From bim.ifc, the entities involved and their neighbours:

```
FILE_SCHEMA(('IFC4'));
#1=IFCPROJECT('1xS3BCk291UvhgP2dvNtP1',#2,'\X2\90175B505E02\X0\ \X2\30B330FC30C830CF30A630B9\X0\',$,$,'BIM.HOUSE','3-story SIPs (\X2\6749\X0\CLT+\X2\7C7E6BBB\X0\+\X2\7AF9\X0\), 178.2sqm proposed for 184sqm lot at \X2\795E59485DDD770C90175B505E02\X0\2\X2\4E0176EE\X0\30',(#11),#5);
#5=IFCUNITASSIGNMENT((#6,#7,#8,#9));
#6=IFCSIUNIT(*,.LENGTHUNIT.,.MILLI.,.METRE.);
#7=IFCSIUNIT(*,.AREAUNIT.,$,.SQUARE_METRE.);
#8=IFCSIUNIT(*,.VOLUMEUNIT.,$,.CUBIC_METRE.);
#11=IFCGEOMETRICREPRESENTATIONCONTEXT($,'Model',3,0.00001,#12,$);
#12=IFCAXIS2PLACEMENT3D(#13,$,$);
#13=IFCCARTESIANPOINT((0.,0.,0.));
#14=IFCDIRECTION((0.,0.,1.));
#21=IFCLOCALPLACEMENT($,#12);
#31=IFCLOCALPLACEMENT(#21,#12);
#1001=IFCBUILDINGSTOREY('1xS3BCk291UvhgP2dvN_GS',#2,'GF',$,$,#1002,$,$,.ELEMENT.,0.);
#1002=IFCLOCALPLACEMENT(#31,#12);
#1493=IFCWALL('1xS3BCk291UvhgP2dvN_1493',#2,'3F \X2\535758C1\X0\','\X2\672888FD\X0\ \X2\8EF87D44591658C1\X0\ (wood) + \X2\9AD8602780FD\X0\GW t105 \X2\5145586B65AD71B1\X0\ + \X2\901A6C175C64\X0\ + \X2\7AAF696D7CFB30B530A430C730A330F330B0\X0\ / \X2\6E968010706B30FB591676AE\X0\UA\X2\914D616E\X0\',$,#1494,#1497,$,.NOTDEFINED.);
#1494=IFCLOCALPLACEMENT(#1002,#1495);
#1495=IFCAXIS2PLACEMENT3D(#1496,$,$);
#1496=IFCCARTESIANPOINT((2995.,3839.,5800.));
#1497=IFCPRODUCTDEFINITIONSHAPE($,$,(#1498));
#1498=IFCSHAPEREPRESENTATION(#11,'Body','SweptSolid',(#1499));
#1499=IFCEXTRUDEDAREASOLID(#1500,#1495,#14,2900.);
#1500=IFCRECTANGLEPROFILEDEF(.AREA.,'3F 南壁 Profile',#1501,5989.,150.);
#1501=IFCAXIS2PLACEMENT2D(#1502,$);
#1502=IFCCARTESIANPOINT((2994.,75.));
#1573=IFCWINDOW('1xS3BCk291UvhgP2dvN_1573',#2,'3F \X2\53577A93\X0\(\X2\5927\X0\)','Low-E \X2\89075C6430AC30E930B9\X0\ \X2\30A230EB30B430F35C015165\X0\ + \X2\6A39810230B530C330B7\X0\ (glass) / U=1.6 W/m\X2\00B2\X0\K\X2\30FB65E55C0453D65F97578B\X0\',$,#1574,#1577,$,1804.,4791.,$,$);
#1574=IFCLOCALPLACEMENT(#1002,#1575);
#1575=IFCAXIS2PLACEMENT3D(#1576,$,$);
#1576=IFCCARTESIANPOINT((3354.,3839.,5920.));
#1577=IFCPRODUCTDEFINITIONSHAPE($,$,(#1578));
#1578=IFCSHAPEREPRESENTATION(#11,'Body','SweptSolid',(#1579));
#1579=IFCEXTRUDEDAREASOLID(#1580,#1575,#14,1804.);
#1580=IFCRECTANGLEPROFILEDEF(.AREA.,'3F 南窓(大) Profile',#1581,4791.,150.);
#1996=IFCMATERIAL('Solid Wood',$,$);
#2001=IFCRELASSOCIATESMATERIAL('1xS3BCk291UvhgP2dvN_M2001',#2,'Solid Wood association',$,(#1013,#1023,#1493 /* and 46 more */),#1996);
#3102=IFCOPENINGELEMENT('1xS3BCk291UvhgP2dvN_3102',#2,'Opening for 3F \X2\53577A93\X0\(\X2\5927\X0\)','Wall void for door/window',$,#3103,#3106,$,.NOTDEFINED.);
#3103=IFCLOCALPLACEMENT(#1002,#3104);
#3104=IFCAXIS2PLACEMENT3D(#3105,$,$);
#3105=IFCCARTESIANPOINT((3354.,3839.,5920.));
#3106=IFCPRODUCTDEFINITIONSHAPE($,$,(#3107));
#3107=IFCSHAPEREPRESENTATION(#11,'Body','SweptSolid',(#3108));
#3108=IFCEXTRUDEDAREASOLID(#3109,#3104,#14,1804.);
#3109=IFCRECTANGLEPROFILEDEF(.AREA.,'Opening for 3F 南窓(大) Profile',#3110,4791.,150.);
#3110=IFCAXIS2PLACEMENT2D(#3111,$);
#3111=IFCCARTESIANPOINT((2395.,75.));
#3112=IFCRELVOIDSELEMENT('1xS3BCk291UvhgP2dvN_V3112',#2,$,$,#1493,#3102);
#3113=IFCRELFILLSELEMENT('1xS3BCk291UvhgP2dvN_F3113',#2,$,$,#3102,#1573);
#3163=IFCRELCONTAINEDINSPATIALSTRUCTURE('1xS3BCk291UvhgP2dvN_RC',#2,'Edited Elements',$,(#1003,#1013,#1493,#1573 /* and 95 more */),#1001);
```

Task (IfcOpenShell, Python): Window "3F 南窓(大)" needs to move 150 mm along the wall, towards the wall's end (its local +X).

```python
import ifcopenshell
import ifcopenshell.api.geometry
import ifcopenshell.util.placement
import ifcopenshell.util.unit

model = ifcopenshell.open("bim.ifc")
unit_scale = ifcopenshell.util.unit.calculate_unit_scale(model)

window = model.by_guid("1xS3BCk291UvhgP2dvN_1573")
opening = window.FillsVoids[0].RelatingOpeningElement
wall = opening.VoidsElements[0].RelatingBuildingElement

wall_matrix = ifcopenshell.util.placement.get_local_placement(wall.ObjectPlacement)
shift = wall_matrix[:3, 0] * 0.15 / unit_scale
before = ifcopenshell.util.placement.get_local_placement(window.ObjectPlacement)[:3, 3].copy()

# The window is not placed relative to its opening, so move both.
for product in (opening, window):
    matrix = ifcopenshell.util.placement.get_local_placement(product.ObjectPlacement)
    matrix[:3, 3] += shift
    ifcopenshell.api.geometry.edit_object_placement(model, product=product, matrix=matrix, is_si=False)

after = ifcopenshell.util.placement.get_local_placement(window.ObjectPlacement)[:3, 3]
print("window moved by", (after - before).round(3) + 0.0)

model.write("bim_v2.ifc")
```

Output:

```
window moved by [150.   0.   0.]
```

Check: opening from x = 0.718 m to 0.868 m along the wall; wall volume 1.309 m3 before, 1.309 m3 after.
